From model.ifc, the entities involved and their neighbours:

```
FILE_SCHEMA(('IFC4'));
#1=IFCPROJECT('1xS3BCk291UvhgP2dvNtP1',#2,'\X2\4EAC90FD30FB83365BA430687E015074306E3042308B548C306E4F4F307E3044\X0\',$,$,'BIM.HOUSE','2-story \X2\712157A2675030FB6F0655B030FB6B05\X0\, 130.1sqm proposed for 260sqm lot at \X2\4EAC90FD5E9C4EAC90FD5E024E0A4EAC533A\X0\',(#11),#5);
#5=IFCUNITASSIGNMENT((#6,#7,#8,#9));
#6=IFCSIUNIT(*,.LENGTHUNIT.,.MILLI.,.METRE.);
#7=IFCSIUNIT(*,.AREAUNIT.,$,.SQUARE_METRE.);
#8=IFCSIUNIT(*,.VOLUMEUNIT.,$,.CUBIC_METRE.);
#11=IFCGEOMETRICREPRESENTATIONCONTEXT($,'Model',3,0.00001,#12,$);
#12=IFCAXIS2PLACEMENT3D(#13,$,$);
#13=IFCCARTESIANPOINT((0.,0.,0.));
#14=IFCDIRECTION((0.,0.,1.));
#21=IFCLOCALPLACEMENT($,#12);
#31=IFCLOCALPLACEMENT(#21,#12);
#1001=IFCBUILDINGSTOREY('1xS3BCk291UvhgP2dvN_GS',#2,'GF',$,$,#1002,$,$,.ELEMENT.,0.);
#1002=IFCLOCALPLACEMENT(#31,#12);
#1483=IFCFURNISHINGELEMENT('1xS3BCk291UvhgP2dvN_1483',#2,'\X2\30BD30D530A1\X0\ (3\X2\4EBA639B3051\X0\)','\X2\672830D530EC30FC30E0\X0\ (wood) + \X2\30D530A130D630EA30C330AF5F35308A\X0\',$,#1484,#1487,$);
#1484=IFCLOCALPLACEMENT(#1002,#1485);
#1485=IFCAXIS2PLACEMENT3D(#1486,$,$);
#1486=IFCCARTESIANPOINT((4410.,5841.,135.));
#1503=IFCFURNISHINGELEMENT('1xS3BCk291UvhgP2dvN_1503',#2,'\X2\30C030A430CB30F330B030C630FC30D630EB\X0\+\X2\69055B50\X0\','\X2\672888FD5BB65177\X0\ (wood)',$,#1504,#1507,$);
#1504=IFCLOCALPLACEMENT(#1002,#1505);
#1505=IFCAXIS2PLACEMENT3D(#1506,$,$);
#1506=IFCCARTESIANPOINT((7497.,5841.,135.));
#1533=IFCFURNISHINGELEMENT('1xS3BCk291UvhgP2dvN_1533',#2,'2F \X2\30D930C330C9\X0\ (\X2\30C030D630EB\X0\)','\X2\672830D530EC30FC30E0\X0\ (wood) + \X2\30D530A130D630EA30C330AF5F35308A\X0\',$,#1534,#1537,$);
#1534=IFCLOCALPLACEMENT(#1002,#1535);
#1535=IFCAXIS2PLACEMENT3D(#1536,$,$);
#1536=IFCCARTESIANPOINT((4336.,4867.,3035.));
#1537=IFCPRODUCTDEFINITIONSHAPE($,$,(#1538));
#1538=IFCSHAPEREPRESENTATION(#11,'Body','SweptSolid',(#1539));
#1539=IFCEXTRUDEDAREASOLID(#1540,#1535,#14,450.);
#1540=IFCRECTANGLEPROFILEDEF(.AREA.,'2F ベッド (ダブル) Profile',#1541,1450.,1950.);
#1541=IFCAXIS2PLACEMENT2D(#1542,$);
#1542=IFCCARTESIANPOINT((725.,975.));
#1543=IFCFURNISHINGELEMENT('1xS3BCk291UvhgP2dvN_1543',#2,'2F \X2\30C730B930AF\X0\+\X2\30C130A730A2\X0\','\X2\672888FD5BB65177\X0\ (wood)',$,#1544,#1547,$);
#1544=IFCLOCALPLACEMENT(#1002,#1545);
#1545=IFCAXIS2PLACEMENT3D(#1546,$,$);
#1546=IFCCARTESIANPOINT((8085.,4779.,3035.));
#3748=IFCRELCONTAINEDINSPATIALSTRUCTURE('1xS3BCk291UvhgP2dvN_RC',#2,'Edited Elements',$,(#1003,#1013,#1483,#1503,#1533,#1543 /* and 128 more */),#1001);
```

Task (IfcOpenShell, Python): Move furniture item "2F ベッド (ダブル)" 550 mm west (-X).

```python
import ifcopenshell
import ifcopenshell.api.geometry
import ifcopenshell.util.placement

model = ifcopenshell.open("model.ifc")

item = model.by_id(1533)
matrix = ifcopenshell.util.placement.get_local_placement(item.ObjectPlacement)
matrix[0, 3] -= 550.0
ifcopenshell.api.geometry.edit_object_placement(model, product=item, matrix=matrix, is_si=False)

print(ifcopenshell.util.placement.get_local_placement(item.ObjectPlacement).round(3) + 0.0)

model.write("model_edited.ifc")
```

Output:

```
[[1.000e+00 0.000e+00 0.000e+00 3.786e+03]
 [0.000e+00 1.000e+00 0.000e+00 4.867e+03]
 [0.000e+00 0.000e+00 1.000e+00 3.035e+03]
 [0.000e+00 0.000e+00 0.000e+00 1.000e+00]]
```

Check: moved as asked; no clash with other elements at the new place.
